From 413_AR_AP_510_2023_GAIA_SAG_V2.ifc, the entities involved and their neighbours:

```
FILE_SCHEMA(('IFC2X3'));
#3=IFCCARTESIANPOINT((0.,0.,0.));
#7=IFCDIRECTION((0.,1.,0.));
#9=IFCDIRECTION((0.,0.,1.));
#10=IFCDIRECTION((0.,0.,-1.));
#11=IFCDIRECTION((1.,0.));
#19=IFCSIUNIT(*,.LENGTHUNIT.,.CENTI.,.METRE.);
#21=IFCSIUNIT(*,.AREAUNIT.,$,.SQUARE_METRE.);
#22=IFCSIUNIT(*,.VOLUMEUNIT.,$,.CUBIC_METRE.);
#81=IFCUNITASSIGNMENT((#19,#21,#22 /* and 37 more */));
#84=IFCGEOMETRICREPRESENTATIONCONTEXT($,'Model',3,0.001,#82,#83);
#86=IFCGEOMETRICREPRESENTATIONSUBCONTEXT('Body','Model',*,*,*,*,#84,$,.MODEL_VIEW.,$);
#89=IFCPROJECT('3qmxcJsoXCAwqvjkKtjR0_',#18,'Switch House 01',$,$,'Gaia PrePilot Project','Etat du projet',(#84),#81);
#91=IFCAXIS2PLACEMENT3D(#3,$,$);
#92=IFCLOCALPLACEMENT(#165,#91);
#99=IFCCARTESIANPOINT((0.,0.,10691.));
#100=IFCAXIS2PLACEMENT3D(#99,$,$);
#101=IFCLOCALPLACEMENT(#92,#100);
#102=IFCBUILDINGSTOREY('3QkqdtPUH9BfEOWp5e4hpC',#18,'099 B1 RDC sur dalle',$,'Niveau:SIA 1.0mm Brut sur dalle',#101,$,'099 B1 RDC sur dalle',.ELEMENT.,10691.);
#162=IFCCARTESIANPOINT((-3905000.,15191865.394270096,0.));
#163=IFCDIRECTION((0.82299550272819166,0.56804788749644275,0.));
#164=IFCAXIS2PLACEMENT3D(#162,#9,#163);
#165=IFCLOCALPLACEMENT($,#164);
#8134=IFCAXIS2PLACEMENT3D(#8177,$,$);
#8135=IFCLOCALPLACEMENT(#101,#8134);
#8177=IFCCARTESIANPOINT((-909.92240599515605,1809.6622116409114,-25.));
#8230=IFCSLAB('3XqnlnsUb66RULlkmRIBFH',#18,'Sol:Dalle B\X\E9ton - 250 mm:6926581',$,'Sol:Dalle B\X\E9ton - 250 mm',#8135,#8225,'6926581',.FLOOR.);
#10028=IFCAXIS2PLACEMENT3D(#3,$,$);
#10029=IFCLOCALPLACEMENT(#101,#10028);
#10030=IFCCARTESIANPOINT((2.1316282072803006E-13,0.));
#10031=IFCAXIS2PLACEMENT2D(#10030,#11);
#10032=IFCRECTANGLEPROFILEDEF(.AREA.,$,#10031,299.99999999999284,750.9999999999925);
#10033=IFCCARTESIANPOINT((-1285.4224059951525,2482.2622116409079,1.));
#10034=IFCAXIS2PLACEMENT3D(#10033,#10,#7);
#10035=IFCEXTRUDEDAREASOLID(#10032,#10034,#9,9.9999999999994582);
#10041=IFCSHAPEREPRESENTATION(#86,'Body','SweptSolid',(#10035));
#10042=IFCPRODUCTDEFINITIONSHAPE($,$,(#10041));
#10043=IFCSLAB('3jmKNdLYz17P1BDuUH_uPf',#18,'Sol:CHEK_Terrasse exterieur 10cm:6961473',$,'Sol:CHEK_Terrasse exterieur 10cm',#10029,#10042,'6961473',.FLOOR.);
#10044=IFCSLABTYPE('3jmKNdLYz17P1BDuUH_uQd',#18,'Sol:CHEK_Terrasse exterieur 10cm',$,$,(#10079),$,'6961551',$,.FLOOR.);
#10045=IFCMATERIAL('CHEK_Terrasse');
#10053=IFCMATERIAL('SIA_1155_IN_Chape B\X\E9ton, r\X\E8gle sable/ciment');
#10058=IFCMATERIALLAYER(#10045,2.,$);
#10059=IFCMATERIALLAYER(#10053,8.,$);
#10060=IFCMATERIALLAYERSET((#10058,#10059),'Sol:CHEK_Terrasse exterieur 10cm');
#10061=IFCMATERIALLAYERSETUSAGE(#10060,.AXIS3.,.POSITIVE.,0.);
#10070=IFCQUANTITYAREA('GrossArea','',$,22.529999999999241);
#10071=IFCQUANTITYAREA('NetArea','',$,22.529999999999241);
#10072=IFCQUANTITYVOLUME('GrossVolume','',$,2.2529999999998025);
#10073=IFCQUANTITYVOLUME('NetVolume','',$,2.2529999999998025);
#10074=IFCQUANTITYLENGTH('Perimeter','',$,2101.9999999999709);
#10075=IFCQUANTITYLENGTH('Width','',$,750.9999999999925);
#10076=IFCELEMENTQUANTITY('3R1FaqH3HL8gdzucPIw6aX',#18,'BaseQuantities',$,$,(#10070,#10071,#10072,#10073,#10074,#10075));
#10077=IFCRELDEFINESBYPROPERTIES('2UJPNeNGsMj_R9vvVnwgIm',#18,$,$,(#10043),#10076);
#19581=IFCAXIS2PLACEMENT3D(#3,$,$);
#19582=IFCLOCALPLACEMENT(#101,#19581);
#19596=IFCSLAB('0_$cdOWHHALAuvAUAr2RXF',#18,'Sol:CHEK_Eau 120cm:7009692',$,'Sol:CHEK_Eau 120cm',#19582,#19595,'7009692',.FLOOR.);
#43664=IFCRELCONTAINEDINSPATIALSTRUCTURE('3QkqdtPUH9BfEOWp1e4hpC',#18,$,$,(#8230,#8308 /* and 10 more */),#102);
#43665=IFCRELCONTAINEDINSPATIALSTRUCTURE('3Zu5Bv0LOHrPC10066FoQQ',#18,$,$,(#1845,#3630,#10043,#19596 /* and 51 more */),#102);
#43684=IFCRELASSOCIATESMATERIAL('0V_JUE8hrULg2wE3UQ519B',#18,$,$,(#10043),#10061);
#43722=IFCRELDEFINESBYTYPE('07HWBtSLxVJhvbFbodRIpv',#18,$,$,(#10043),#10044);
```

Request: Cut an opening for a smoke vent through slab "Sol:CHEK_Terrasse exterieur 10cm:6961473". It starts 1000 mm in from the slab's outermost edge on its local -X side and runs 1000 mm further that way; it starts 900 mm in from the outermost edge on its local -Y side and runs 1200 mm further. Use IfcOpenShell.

```python
import numpy as np
import ifcopenshell
import ifcopenshell.api.feature
import ifcopenshell.api.geometry
import ifcopenshell.api.pset
import ifcopenshell.api.root
import ifcopenshell.geom
import ifcopenshell.util.element
import ifcopenshell.util.placement
import ifcopenshell.util.representation
import ifcopenshell.util.shape
import ifcopenshell.util.unit

model = ifcopenshell.open("413_AR_AP_510_2023_GAIA_SAG_V2.ifc")
unit_scale = ifcopenshell.util.unit.calculate_unit_scale(model)
area_scale = ifcopenshell.util.unit.calculate_unit_scale(model, "AREAUNIT")
volume_scale = ifcopenshell.util.unit.calculate_unit_scale(model, "VOLUMEUNIT")
settings = ifcopenshell.geom.settings()


def volume(element):
    """Net volume in cubic metres, openings subtracted."""
    shape = ifcopenshell.geom.create_shape(settings, element)
    return ifcopenshell.util.shape.get_volume(shape.geometry)


slab = model.by_guid("3jmKNdLYz17P1BDuUH_uPf")
before = volume(slab)

# Extent in the slab's own axes, in metres. The edges named are its -X and -Y sides.
slab_shape = ifcopenshell.geom.create_shape(settings, slab)
vertices = ifcopenshell.util.shape.get_vertices(slab_shape.geometry)
x_min, y_min, bottom = vertices.min(axis=0)
top = vertices[:, 2].max()

opening = ifcopenshell.api.root.create_entity(model, ifc_class="IfcOpeningElement", name="Smoke vent opening")
context = ifcopenshell.util.representation.get_context(model, "Model", "Body", "MODEL_VIEW")
width, depth = 1, 1.2
outline = [(0.0, 0.0), (width, 0.0), (width, depth), (0.0, depth), (0.0, 0.0)]
# Overshoot both faces by 50 mm so the cut is clean.
shape = ifcopenshell.api.geometry.add_slab_representation(
    model, context=context, depth=top - bottom + 0.1, polyline=outline
)
ifcopenshell.api.geometry.assign_representation(model, product=opening, representation=shape)

matrix = ifcopenshell.util.placement.get_local_placement(slab.ObjectPlacement)
matrix[:, 3] = matrix @ np.append(np.array([x_min + 1, y_min + 0.9, bottom - 0.05]) / unit_scale, 1.0)
ifcopenshell.api.geometry.edit_object_placement(model, product=opening, matrix=matrix, is_si=False)
ifcopenshell.api.feature.add_feature(model, feature=opening, element=slab)

after = volume(slab)

# Update the slab's stored quantities.
qto = model.by_id(ifcopenshell.util.element.get_pset(slab, "BaseQuantities", should_inherit=False)["id"])
ifcopenshell.api.pset.edit_qto(model, qto=qto, properties={
    "NetArea": after / (top - bottom) / area_scale,
    "NetVolume": after / volume_scale,
})

print(f"slab volume {before:.3f} -> {after:.3f} m3")

model.write("413_AR_AP_510_2023_GAIA_SAG_V2_edited.ifc")
```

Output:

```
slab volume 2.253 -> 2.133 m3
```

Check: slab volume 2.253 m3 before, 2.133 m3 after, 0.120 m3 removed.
